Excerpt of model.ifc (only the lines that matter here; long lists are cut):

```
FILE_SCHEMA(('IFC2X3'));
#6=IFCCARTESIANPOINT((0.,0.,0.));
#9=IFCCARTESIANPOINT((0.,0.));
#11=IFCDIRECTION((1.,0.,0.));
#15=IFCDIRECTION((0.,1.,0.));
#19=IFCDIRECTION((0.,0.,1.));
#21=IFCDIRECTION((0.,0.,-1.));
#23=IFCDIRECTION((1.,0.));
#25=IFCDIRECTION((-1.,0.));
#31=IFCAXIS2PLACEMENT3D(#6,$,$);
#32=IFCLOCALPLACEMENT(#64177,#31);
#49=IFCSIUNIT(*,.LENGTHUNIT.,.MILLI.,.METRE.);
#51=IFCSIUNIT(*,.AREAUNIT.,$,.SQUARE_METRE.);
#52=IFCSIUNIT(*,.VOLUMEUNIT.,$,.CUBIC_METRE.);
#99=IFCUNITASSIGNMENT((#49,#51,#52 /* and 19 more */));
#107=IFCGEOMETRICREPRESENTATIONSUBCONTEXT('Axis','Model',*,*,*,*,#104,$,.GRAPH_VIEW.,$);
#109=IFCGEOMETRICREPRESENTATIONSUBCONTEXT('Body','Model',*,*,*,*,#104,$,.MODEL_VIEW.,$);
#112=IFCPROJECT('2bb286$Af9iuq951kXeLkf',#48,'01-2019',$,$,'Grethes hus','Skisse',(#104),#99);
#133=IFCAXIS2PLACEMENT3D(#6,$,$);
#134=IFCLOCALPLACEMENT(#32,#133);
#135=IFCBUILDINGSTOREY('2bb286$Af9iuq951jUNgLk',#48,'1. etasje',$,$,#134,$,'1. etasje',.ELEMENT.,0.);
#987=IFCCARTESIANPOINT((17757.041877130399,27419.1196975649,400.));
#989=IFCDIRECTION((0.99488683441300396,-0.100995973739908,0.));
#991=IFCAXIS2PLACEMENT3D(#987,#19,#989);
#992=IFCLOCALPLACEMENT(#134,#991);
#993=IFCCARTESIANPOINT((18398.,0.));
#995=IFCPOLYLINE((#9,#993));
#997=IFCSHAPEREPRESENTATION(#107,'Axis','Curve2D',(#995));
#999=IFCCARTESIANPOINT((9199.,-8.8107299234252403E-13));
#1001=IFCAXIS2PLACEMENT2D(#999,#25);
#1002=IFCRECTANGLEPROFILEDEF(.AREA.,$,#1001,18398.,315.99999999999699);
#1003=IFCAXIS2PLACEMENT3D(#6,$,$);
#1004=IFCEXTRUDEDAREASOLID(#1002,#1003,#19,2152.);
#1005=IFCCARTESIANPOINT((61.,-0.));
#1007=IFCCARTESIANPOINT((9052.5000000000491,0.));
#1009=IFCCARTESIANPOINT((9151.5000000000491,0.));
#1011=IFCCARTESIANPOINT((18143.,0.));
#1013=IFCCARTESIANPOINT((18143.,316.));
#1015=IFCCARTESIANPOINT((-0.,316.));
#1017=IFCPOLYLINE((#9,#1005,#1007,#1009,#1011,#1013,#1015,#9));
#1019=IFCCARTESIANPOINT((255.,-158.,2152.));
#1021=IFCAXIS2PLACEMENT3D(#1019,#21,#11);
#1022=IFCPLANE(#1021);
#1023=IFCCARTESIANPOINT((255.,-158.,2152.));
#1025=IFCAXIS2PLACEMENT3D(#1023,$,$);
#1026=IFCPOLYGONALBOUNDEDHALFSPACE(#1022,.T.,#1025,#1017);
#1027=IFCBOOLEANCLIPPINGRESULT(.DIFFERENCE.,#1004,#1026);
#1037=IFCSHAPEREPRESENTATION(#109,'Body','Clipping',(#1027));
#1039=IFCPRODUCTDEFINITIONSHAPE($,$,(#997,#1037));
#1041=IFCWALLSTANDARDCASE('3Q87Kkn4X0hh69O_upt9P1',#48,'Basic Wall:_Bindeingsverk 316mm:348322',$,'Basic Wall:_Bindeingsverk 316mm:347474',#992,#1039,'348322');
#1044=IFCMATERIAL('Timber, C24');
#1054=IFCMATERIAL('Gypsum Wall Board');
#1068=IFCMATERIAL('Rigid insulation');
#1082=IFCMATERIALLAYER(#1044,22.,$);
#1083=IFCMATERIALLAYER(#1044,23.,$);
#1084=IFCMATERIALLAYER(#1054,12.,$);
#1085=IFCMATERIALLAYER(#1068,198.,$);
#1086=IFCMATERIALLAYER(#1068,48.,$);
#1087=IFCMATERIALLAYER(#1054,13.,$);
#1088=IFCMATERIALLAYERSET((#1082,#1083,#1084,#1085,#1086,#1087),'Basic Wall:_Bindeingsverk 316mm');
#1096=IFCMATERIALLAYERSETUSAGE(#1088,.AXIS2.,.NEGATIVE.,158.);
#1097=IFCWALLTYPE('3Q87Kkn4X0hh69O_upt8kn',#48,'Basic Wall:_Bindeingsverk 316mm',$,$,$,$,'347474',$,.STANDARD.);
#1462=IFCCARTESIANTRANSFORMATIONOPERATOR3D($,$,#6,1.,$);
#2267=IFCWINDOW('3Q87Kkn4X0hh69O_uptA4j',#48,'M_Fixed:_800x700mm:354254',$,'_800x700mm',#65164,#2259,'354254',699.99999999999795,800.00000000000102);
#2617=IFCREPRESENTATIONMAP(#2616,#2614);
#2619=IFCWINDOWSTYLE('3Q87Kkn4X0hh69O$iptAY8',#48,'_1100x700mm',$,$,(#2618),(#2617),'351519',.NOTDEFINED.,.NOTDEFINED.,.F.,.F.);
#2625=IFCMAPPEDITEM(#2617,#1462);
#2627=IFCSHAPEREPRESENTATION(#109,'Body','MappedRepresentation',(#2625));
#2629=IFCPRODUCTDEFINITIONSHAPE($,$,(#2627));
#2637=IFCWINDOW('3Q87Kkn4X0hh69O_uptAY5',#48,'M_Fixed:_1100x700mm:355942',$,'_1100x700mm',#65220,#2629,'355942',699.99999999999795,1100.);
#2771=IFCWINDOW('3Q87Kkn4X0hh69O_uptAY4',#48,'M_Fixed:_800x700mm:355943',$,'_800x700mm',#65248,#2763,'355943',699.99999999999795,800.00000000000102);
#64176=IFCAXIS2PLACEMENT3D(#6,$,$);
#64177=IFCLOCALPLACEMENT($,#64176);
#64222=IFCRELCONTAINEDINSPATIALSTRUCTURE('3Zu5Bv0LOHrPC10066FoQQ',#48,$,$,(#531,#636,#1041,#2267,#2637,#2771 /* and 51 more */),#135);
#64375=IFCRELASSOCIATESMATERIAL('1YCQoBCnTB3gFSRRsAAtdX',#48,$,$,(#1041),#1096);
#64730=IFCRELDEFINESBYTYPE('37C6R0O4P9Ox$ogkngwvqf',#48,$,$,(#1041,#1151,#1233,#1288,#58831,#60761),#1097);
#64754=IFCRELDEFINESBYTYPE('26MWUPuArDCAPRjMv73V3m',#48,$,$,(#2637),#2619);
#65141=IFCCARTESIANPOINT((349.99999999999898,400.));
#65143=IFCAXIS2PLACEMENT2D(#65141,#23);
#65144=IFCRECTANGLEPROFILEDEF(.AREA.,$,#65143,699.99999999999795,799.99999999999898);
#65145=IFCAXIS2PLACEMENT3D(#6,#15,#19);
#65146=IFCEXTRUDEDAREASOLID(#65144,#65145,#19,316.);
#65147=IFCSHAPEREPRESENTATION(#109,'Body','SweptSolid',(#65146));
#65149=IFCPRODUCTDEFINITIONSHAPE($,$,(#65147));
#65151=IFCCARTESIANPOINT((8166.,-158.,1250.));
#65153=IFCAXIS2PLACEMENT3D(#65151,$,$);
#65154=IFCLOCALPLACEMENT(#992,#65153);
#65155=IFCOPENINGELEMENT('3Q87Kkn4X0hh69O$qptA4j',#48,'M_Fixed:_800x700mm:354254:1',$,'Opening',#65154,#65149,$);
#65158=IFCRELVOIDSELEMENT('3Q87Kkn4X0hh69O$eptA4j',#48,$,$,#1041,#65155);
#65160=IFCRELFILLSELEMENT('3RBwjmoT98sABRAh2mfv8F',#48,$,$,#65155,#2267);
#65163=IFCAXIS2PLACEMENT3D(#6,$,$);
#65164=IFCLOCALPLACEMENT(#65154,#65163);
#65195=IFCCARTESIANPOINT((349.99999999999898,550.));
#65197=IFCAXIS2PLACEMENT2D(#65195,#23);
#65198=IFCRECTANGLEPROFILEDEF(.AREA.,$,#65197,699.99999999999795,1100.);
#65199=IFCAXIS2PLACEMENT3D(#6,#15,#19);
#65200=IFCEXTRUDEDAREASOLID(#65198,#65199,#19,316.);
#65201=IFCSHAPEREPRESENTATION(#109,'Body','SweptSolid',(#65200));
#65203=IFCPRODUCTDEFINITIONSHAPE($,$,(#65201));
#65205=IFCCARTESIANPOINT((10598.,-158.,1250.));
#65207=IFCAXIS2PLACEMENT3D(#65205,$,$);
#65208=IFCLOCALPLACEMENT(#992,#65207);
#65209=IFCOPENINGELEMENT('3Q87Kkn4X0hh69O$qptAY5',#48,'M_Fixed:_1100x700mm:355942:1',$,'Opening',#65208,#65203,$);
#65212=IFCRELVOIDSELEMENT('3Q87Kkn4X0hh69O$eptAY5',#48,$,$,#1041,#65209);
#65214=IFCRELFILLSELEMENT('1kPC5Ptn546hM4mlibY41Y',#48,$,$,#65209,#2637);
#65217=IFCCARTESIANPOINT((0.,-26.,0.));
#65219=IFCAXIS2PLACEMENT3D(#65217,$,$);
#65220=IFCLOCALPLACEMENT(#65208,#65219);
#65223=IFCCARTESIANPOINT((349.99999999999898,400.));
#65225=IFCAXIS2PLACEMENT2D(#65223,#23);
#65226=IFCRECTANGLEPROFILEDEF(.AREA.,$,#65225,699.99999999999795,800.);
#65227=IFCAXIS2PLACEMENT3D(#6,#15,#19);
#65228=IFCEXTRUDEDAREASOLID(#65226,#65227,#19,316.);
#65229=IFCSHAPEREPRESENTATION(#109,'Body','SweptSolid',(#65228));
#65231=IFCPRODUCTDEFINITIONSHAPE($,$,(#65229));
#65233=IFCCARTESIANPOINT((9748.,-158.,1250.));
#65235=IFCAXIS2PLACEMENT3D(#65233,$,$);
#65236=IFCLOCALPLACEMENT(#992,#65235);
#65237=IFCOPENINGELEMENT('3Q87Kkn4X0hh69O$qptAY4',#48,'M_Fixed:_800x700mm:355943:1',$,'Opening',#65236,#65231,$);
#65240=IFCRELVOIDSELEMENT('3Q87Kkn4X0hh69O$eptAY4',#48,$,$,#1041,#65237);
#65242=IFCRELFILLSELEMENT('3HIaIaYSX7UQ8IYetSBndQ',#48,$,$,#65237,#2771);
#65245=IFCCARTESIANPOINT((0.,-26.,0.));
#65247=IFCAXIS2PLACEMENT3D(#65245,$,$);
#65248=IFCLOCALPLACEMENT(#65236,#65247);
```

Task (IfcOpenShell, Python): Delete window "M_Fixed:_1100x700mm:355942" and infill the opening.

```python
import ifcopenshell
import ifcopenshell.api.feature
import ifcopenshell.api.root
import ifcopenshell.geom
import ifcopenshell.util.shape

model = ifcopenshell.open("model.ifc")
settings = ifcopenshell.geom.settings()


def volume(element):
    """Net volume in cubic metres, openings subtracted."""
    shape = ifcopenshell.geom.create_shape(settings, element)
    return ifcopenshell.util.shape.get_volume(shape.geometry)


window = model.by_guid("3Q87Kkn4X0hh69O_uptAY5")
opening = window.FillsVoids[0].RelatingOpeningElement
wall = opening.VoidsElements[0].RelatingBuildingElement
before = volume(wall)

ifcopenshell.api.root.remove_product(model, product=window)
ifcopenshell.api.feature.remove_feature(model, feature=opening)

after = volume(wall)

print(f"wall volume {before:.3f} -> {after:.3f} m3")

model.write("model_updated.ifc")
```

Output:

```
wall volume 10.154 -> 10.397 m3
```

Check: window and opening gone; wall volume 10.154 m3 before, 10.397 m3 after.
